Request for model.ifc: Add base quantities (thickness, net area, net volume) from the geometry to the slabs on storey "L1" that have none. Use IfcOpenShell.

First a look at what the model holds.

```python
import ifcopenshell
import ifcopenshell.util.element
import ifcopenshell.util.unit

model = ifcopenshell.open("model.ifc")
print(model.schema)
for unit_type in ("LENGTHUNIT", "AREAUNIT", "VOLUMEUNIT"):
    print(unit_type, ifcopenshell.util.unit.calculate_unit_scale(model, unit_type))
storey = next(s for s in model.by_type("IfcBuildingStorey") if s.Name == "L1")
slabs = [e for e in ifcopenshell.util.element.get_decomposition(storey) if e.is_a("IfcSlab")]
for e in sorted(slabs, key=lambda e: e.id()):
    print(e.id(), e.is_a(), e.Name, list(ifcopenshell.util.element.get_psets(e, qtos_only=True)), sep=" | ")
```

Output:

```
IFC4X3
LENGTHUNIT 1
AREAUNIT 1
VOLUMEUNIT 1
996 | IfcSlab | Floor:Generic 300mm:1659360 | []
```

```python
import ifcopenshell
import ifcopenshell.api.pset
import ifcopenshell.geom
import ifcopenshell.util.element
import ifcopenshell.util.shape
import ifcopenshell.util.unit

model = ifcopenshell.open("model.ifc")
unit_scale = ifcopenshell.util.unit.calculate_unit_scale(model)
area_scale = ifcopenshell.util.unit.calculate_unit_scale(model, "AREAUNIT")
volume_scale = ifcopenshell.util.unit.calculate_unit_scale(model, "VOLUMEUNIT")
settings = ifcopenshell.geom.settings()

storey = next(s for s in model.by_type("IfcBuildingStorey") if s.Name == "L1")
slabs = [e for e in ifcopenshell.util.element.get_decomposition(storey) if e.is_a("IfcSlab")]

for e in sorted(slabs, key=lambda e: e.id()):
    if ifcopenshell.util.element.get_psets(e, qtos_only=True, should_inherit=False):
        continue
    # Geometry comes back in metres, in the element's own axes.
    shape = ifcopenshell.geom.create_shape(settings, e)
    values = {
        "Width": ifcopenshell.util.shape.get_z(shape.geometry) / unit_scale,
        "NetArea": ifcopenshell.util.shape.get_footprint_area(shape.geometry) / area_scale,
        "NetVolume": ifcopenshell.util.shape.get_volume(shape.geometry) / volume_scale,
    }
    qto = ifcopenshell.api.pset.add_qto(model, product=e, name="Qto_SlabBaseQuantities")
    ifcopenshell.api.pset.edit_qto(model, qto=qto, properties=values)
    print(e.id(), {k: round(v, 3) for k, v in values.items()})

model.write("model-out.ifc")
```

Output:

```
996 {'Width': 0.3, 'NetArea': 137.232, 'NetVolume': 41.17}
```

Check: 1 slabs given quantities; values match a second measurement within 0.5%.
